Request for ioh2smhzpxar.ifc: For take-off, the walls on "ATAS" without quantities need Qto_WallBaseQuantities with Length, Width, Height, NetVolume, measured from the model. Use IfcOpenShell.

First a look at what the model holds.

```python
import ifcopenshell
import ifcopenshell.util.element
import ifcopenshell.util.unit

model = ifcopenshell.open("ioh2smhzpxar.ifc")
print(model.schema)
for unit_type in ("LENGTHUNIT", "AREAUNIT", "VOLUMEUNIT"):
    print(unit_type, ifcopenshell.util.unit.calculate_unit_scale(model, unit_type))
storey = next(s for s in model.by_type("IfcBuildingStorey") if s.Name == "ATAS")
walls = [e for e in ifcopenshell.util.element.get_decomposition(storey) if e.is_a("IfcWall")]
for e in sorted(walls, key=lambda e: e.id()):
    print(e.id(), e.is_a(), e.Name, list(ifcopenshell.util.element.get_psets(e, qtos_only=True)), sep=" | ")
```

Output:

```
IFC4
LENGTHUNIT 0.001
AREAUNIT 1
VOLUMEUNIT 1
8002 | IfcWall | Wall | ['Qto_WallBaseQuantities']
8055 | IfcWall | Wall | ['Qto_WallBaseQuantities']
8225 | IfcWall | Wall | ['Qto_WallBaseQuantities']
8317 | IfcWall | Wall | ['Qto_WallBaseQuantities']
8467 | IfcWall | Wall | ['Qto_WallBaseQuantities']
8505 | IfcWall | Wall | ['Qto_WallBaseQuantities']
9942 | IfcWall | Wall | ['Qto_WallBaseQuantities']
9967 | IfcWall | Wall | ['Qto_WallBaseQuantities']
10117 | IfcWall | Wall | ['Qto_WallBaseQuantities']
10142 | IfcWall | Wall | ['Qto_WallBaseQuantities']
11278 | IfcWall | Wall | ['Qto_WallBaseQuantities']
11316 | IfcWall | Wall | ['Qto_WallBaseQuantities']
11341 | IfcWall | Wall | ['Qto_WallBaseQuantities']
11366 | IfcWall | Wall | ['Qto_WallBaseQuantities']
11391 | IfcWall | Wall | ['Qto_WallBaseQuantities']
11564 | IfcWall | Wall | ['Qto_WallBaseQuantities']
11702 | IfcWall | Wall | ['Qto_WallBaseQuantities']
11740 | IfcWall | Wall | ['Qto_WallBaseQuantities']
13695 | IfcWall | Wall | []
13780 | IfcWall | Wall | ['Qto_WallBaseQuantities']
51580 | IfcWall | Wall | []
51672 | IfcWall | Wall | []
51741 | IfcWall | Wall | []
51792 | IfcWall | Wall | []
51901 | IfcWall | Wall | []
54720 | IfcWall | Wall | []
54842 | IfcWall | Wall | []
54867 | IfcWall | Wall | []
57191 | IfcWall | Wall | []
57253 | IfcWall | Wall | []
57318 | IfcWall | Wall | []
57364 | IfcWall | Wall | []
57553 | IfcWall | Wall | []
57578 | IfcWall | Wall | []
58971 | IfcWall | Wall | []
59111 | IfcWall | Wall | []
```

```python
import ifcopenshell
import ifcopenshell.api.pset
import ifcopenshell.geom
import ifcopenshell.util.element
import ifcopenshell.util.shape
import ifcopenshell.util.unit

model = ifcopenshell.open("ioh2smhzpxar.ifc")
unit_scale = ifcopenshell.util.unit.calculate_unit_scale(model)
volume_scale = ifcopenshell.util.unit.calculate_unit_scale(model, "VOLUMEUNIT")
settings = ifcopenshell.geom.settings()

storey = next(s for s in model.by_type("IfcBuildingStorey") if s.Name == "ATAS")
walls = [e for e in ifcopenshell.util.element.get_decomposition(storey) if e.is_a("IfcWall")]

for e in sorted(walls, key=lambda e: e.id()):
    if ifcopenshell.util.element.get_psets(e, qtos_only=True, should_inherit=False):
        continue
    # Geometry comes back in metres, in the element's own axes.
    shape = ifcopenshell.geom.create_shape(settings, e)
    values = {
        "Length": ifcopenshell.util.shape.get_x(shape.geometry) / unit_scale,
        "Width": ifcopenshell.util.shape.get_y(shape.geometry) / unit_scale,
        "Height": ifcopenshell.util.shape.get_z(shape.geometry) / unit_scale,
        "NetVolume": ifcopenshell.util.shape.get_volume(shape.geometry) / volume_scale,
    }
    qto = ifcopenshell.api.pset.add_qto(model, product=e, name="Qto_WallBaseQuantities")
    ifcopenshell.api.pset.edit_qto(model, qto=qto, properties=values)
    print(e.id(), {k: round(v, 3) for k, v in values.items()})

model.write("ioh2smhzpxar-out.ifc")
```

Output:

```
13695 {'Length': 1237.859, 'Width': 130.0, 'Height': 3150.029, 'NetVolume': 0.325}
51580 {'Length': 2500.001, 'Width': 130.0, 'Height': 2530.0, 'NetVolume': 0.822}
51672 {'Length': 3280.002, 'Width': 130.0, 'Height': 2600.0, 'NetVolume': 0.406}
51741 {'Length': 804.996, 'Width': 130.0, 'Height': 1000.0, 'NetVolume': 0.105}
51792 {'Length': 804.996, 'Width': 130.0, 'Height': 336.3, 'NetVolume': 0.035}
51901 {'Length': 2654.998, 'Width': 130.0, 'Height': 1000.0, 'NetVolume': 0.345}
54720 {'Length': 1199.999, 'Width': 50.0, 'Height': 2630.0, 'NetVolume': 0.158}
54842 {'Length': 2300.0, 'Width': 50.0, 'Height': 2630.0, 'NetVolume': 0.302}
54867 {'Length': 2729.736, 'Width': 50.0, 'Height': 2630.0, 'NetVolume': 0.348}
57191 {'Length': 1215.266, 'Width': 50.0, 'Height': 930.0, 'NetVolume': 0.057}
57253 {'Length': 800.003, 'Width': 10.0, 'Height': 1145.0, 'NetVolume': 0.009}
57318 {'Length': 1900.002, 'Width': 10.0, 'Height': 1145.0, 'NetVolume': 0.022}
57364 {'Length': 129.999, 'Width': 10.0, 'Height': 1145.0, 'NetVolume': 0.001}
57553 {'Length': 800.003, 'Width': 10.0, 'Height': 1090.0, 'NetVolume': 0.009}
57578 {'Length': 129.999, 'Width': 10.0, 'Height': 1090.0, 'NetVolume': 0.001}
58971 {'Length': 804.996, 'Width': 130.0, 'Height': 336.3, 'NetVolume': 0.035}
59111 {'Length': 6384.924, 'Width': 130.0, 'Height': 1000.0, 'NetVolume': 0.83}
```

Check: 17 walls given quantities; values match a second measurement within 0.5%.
